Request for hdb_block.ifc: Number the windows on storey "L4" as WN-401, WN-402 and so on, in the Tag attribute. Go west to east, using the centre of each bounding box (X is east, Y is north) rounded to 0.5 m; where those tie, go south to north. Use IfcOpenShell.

First a look at what the model holds.

```python
import ifcopenshell
import ifcopenshell.util.element
import ifcopenshell.util.placement

model = ifcopenshell.open("hdb_block.ifc")
print(model.schema)
storey = next(s for s in model.by_type("IfcBuildingStorey") if s.Name == "L4")
windows = [e for e in ifcopenshell.util.element.get_decomposition(storey) if e.is_a("IfcWindow")]
for e in sorted(windows, key=lambda e: e.id()):
    origin = ifcopenshell.util.placement.get_local_placement(e.ObjectPlacement)[:3, 3]
    print(e.id(), e.Tag, e.Name, origin.round(2) + 0.0, sep=" | ")
```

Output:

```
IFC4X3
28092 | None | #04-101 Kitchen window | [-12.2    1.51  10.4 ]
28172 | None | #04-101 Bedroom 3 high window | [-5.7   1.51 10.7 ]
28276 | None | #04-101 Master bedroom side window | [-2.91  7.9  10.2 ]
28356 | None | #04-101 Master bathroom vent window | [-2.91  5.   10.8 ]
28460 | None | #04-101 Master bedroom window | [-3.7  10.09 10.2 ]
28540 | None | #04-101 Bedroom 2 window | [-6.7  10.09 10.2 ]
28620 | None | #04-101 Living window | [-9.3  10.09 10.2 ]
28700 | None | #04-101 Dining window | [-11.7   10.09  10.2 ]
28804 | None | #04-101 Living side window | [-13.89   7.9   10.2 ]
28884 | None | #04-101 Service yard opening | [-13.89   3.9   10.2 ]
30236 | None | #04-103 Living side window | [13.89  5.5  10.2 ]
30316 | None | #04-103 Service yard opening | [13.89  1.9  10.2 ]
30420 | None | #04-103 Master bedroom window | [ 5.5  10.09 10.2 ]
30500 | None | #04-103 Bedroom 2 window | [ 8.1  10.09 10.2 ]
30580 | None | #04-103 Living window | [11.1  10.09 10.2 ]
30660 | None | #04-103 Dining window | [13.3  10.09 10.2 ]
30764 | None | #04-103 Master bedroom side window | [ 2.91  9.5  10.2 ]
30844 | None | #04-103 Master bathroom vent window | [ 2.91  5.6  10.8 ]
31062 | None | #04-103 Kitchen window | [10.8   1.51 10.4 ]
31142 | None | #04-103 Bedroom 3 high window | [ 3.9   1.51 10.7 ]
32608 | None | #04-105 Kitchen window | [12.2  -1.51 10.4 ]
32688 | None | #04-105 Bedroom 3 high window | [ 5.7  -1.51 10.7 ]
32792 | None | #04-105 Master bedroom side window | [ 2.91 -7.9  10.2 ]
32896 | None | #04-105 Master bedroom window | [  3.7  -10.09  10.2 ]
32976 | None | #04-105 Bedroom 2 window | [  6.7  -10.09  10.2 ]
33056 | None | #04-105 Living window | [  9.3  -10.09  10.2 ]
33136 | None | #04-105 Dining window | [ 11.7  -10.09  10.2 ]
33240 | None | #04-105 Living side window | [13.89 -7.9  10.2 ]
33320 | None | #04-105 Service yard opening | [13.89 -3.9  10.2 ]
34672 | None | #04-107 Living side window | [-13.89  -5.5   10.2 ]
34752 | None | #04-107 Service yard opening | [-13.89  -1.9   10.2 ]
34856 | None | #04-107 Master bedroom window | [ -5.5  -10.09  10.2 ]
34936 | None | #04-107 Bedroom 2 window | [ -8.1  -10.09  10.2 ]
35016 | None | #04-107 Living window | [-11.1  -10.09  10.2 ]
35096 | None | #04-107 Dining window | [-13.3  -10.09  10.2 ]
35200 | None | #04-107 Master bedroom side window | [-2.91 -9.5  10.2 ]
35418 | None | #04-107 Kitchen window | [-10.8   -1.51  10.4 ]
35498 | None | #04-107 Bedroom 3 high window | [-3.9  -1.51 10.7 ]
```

```python
import ifcopenshell
import ifcopenshell.geom
import ifcopenshell.util.element
import ifcopenshell.util.shape

model = ifcopenshell.open("hdb_block.ifc")
settings = ifcopenshell.geom.settings()
settings.set("use-world-coords", True)


def centre(element):
    shape = ifcopenshell.geom.create_shape(settings, element)
    return ifcopenshell.util.shape.get_bbox_centroid(shape.geometry)


storey = next(s for s in model.by_type("IfcBuildingStorey") if s.Name == "L4")
windows = [e for e in ifcopenshell.util.element.get_decomposition(storey) if e.is_a("IfcWindow")]

# Insertion points can sit at a corner or the storey origin, so sort by the geometry (in metres).
centres = {e: centre(e) for e in windows}
windows.sort(key=lambda e: (round(centres[e][0] / 0.5), centres[e][1]))

for i, e in enumerate(windows, start=1):
    number = f"WN-4{i:02d}"
    e.Tag = number
    print(e.id(), number)

model.write("hdb_block_updated.ifc")
```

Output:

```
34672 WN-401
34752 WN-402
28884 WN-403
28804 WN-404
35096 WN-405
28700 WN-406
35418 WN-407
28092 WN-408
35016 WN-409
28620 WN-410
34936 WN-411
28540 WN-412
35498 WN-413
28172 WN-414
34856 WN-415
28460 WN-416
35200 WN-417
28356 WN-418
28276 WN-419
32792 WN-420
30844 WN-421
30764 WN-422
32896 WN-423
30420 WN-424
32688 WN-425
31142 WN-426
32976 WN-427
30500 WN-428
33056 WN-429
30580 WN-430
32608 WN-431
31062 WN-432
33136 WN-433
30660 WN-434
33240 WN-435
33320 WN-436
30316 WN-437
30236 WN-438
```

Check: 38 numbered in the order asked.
